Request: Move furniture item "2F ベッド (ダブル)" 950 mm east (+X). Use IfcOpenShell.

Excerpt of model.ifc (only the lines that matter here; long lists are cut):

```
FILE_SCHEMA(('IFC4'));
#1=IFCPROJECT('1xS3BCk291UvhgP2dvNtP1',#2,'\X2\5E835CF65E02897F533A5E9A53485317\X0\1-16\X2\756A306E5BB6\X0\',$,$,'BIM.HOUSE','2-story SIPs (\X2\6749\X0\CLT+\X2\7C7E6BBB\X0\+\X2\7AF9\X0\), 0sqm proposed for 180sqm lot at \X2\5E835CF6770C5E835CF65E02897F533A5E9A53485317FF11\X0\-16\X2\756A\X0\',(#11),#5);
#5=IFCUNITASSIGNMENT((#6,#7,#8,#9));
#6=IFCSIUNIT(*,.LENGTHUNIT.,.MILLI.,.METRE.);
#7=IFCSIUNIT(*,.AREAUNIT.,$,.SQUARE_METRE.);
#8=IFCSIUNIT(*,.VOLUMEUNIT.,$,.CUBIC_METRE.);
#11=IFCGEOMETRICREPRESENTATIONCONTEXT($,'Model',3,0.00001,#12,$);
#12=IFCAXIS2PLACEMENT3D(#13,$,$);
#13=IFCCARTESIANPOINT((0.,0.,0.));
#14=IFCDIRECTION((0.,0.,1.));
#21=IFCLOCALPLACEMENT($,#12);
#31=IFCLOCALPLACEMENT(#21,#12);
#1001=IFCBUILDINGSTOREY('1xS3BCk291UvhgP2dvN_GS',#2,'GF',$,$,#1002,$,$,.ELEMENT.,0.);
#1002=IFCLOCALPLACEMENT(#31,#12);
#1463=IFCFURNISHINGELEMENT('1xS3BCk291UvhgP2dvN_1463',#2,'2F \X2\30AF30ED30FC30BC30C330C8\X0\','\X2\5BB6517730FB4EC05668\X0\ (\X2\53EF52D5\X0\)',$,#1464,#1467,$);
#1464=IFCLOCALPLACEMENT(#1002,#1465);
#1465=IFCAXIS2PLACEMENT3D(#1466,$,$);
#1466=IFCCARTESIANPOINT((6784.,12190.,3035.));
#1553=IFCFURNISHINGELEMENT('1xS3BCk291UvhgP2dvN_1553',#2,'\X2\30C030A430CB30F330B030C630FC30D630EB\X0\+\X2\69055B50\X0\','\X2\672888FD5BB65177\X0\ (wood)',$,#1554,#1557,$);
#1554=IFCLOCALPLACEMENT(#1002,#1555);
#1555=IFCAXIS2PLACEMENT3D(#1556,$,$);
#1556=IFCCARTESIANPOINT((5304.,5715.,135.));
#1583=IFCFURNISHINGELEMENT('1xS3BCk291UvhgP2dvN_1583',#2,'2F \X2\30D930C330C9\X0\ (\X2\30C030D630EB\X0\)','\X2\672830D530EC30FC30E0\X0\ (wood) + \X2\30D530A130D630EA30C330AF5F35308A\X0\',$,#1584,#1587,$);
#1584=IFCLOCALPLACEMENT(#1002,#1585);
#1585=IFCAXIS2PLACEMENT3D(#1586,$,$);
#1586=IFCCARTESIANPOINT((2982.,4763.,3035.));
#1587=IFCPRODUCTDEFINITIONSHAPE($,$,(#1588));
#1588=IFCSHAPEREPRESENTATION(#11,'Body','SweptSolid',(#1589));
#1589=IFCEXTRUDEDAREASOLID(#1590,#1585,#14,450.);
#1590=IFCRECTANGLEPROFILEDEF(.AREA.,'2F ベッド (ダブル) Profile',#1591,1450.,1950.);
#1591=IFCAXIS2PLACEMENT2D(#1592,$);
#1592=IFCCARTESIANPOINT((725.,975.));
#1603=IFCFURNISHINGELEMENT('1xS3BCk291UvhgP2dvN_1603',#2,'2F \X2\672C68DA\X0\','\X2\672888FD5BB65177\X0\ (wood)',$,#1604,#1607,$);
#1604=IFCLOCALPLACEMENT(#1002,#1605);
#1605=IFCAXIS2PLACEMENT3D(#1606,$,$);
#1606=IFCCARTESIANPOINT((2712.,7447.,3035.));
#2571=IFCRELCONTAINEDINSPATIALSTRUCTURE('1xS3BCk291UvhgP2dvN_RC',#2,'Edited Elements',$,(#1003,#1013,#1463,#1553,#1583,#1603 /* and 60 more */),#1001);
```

```python
import ifcopenshell
import ifcopenshell.api.geometry
import ifcopenshell.util.placement

model = ifcopenshell.open("model.ifc")

item = model.by_id(1583)
matrix = ifcopenshell.util.placement.get_local_placement(item.ObjectPlacement)
matrix[0, 3] += 950.0
ifcopenshell.api.geometry.edit_object_placement(model, product=item, matrix=matrix, is_si=False)

print(ifcopenshell.util.placement.get_local_placement(item.ObjectPlacement).round(3) + 0.0)

model.write("model-out.ifc")
```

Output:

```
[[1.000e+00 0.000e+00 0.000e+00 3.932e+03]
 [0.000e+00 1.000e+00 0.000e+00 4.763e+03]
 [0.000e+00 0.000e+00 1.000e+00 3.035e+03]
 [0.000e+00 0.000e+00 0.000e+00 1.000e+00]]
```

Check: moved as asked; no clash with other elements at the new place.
